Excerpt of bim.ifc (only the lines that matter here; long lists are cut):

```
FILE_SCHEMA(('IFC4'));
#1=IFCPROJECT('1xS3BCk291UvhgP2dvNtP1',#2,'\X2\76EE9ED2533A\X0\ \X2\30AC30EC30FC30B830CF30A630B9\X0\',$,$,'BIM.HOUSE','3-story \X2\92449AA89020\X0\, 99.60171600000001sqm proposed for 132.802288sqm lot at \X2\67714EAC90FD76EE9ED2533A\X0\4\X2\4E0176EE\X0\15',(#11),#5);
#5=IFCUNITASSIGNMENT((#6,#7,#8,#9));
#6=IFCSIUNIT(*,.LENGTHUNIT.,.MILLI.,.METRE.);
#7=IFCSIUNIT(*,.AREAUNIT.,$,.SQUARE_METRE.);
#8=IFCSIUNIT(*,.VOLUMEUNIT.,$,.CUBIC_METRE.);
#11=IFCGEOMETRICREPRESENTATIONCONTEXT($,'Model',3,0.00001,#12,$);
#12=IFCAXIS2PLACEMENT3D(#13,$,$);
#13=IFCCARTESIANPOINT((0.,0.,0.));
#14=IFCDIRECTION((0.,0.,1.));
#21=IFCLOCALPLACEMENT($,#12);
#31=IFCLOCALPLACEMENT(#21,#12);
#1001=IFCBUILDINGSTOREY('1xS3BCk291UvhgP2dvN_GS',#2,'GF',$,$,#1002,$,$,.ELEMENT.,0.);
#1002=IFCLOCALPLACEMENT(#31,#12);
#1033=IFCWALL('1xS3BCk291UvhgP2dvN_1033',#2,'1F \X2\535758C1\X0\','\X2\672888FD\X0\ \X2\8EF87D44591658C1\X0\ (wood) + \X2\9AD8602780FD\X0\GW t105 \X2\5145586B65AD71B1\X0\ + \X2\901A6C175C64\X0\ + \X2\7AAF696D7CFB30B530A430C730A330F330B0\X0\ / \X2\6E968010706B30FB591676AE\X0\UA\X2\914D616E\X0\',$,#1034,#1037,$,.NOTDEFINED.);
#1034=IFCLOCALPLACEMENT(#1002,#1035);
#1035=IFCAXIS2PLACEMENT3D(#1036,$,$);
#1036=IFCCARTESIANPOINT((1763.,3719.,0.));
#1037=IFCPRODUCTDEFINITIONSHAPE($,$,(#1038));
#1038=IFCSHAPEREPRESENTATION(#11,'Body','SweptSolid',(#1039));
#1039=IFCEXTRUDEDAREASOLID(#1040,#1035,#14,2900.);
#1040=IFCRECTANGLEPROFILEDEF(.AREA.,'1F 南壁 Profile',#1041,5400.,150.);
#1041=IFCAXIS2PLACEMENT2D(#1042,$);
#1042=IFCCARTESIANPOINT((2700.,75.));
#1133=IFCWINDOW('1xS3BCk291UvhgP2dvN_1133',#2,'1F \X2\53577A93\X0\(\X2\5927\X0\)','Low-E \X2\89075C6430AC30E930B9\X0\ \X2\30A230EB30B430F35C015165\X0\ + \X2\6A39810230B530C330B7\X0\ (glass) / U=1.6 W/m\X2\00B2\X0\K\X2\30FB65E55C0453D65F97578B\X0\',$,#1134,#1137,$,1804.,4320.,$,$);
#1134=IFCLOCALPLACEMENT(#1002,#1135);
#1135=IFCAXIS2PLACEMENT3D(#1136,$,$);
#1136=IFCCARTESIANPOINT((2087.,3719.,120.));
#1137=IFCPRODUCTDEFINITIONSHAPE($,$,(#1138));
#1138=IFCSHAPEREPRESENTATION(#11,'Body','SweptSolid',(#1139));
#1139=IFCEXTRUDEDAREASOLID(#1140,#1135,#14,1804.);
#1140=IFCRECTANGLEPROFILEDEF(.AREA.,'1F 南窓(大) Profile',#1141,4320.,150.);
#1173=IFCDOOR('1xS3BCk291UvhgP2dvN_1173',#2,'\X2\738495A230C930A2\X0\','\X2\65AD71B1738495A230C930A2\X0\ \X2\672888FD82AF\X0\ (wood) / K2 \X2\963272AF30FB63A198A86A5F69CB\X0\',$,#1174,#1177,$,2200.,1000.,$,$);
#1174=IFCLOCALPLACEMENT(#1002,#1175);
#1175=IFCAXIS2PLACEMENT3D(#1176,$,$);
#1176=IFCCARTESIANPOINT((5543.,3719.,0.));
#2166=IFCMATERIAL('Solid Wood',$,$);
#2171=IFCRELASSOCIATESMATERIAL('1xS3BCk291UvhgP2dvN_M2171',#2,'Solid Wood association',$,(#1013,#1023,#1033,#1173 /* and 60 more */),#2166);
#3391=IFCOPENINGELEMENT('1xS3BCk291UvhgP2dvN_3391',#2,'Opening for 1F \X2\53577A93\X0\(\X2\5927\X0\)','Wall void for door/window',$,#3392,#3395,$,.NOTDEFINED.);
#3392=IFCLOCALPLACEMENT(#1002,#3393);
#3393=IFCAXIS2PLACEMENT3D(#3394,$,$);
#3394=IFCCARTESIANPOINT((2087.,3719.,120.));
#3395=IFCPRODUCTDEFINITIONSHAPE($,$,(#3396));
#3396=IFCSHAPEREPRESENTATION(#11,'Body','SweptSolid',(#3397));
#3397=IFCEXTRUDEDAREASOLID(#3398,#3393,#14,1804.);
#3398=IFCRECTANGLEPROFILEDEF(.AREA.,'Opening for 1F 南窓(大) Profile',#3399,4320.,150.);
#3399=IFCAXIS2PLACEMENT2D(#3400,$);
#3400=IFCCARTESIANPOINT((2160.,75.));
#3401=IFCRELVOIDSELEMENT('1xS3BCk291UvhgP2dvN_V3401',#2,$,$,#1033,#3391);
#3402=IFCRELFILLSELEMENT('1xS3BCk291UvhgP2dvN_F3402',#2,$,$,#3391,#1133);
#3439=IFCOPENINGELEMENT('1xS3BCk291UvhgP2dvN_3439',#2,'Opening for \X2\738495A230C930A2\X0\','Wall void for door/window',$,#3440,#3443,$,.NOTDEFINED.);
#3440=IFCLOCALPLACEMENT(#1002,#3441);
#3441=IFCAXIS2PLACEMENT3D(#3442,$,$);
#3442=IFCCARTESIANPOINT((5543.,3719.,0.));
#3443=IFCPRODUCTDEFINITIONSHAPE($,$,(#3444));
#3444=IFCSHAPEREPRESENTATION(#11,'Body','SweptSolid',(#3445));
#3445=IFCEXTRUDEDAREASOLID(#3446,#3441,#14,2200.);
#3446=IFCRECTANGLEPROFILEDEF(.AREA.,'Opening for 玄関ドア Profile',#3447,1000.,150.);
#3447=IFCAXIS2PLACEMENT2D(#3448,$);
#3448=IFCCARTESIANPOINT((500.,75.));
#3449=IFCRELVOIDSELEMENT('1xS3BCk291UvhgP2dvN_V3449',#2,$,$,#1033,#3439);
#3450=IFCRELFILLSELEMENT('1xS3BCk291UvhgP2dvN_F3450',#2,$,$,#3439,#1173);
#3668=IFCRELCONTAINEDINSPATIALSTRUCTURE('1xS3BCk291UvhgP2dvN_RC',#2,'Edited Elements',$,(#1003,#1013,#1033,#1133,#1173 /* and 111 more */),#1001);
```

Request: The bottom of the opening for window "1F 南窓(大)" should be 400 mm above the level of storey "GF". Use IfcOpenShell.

```python
import numpy as np
import ifcopenshell
import ifcopenshell.api.geometry
import ifcopenshell.geom
import ifcopenshell.util.element
import ifcopenshell.util.placement
import ifcopenshell.util.shape
import ifcopenshell.util.unit

model = ifcopenshell.open("bim.ifc")
unit_scale = ifcopenshell.util.unit.calculate_unit_scale(model)

window = model.by_guid("1xS3BCk291UvhgP2dvN_1133")
opening = window.FillsVoids[0].RelatingOpeningElement
storey = ifcopenshell.util.element.get_container(window, ifc_class="IfcBuildingStorey")
level = ifcopenshell.util.placement.get_local_placement(storey.ObjectPlacement)[2, 3]

# The opening's origin need not be at the sill, so measure its lowest point.
shape = ifcopenshell.geom.create_shape(ifcopenshell.geom.settings(), opening)
bottom = ifcopenshell.util.shape.get_shape_bottom_elevation(shape, shape.geometry) / unit_scale
dz = level + 0.4 / unit_scale - bottom

shift = np.array([0.0, 0.0, dz])
# The window is not placed relative to its opening, so move both.
for product in (opening, window):
    matrix = ifcopenshell.util.placement.get_local_placement(product.ObjectPlacement)
    matrix[:3, 3] += shift
    ifcopenshell.api.geometry.edit_object_placement(model, product=product, matrix=matrix, is_si=False)

print(f"moved by {dz * unit_scale:+.3f} m")

model.write("bim_v2.ifc")
```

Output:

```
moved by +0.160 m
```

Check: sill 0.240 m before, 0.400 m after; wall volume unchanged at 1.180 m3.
